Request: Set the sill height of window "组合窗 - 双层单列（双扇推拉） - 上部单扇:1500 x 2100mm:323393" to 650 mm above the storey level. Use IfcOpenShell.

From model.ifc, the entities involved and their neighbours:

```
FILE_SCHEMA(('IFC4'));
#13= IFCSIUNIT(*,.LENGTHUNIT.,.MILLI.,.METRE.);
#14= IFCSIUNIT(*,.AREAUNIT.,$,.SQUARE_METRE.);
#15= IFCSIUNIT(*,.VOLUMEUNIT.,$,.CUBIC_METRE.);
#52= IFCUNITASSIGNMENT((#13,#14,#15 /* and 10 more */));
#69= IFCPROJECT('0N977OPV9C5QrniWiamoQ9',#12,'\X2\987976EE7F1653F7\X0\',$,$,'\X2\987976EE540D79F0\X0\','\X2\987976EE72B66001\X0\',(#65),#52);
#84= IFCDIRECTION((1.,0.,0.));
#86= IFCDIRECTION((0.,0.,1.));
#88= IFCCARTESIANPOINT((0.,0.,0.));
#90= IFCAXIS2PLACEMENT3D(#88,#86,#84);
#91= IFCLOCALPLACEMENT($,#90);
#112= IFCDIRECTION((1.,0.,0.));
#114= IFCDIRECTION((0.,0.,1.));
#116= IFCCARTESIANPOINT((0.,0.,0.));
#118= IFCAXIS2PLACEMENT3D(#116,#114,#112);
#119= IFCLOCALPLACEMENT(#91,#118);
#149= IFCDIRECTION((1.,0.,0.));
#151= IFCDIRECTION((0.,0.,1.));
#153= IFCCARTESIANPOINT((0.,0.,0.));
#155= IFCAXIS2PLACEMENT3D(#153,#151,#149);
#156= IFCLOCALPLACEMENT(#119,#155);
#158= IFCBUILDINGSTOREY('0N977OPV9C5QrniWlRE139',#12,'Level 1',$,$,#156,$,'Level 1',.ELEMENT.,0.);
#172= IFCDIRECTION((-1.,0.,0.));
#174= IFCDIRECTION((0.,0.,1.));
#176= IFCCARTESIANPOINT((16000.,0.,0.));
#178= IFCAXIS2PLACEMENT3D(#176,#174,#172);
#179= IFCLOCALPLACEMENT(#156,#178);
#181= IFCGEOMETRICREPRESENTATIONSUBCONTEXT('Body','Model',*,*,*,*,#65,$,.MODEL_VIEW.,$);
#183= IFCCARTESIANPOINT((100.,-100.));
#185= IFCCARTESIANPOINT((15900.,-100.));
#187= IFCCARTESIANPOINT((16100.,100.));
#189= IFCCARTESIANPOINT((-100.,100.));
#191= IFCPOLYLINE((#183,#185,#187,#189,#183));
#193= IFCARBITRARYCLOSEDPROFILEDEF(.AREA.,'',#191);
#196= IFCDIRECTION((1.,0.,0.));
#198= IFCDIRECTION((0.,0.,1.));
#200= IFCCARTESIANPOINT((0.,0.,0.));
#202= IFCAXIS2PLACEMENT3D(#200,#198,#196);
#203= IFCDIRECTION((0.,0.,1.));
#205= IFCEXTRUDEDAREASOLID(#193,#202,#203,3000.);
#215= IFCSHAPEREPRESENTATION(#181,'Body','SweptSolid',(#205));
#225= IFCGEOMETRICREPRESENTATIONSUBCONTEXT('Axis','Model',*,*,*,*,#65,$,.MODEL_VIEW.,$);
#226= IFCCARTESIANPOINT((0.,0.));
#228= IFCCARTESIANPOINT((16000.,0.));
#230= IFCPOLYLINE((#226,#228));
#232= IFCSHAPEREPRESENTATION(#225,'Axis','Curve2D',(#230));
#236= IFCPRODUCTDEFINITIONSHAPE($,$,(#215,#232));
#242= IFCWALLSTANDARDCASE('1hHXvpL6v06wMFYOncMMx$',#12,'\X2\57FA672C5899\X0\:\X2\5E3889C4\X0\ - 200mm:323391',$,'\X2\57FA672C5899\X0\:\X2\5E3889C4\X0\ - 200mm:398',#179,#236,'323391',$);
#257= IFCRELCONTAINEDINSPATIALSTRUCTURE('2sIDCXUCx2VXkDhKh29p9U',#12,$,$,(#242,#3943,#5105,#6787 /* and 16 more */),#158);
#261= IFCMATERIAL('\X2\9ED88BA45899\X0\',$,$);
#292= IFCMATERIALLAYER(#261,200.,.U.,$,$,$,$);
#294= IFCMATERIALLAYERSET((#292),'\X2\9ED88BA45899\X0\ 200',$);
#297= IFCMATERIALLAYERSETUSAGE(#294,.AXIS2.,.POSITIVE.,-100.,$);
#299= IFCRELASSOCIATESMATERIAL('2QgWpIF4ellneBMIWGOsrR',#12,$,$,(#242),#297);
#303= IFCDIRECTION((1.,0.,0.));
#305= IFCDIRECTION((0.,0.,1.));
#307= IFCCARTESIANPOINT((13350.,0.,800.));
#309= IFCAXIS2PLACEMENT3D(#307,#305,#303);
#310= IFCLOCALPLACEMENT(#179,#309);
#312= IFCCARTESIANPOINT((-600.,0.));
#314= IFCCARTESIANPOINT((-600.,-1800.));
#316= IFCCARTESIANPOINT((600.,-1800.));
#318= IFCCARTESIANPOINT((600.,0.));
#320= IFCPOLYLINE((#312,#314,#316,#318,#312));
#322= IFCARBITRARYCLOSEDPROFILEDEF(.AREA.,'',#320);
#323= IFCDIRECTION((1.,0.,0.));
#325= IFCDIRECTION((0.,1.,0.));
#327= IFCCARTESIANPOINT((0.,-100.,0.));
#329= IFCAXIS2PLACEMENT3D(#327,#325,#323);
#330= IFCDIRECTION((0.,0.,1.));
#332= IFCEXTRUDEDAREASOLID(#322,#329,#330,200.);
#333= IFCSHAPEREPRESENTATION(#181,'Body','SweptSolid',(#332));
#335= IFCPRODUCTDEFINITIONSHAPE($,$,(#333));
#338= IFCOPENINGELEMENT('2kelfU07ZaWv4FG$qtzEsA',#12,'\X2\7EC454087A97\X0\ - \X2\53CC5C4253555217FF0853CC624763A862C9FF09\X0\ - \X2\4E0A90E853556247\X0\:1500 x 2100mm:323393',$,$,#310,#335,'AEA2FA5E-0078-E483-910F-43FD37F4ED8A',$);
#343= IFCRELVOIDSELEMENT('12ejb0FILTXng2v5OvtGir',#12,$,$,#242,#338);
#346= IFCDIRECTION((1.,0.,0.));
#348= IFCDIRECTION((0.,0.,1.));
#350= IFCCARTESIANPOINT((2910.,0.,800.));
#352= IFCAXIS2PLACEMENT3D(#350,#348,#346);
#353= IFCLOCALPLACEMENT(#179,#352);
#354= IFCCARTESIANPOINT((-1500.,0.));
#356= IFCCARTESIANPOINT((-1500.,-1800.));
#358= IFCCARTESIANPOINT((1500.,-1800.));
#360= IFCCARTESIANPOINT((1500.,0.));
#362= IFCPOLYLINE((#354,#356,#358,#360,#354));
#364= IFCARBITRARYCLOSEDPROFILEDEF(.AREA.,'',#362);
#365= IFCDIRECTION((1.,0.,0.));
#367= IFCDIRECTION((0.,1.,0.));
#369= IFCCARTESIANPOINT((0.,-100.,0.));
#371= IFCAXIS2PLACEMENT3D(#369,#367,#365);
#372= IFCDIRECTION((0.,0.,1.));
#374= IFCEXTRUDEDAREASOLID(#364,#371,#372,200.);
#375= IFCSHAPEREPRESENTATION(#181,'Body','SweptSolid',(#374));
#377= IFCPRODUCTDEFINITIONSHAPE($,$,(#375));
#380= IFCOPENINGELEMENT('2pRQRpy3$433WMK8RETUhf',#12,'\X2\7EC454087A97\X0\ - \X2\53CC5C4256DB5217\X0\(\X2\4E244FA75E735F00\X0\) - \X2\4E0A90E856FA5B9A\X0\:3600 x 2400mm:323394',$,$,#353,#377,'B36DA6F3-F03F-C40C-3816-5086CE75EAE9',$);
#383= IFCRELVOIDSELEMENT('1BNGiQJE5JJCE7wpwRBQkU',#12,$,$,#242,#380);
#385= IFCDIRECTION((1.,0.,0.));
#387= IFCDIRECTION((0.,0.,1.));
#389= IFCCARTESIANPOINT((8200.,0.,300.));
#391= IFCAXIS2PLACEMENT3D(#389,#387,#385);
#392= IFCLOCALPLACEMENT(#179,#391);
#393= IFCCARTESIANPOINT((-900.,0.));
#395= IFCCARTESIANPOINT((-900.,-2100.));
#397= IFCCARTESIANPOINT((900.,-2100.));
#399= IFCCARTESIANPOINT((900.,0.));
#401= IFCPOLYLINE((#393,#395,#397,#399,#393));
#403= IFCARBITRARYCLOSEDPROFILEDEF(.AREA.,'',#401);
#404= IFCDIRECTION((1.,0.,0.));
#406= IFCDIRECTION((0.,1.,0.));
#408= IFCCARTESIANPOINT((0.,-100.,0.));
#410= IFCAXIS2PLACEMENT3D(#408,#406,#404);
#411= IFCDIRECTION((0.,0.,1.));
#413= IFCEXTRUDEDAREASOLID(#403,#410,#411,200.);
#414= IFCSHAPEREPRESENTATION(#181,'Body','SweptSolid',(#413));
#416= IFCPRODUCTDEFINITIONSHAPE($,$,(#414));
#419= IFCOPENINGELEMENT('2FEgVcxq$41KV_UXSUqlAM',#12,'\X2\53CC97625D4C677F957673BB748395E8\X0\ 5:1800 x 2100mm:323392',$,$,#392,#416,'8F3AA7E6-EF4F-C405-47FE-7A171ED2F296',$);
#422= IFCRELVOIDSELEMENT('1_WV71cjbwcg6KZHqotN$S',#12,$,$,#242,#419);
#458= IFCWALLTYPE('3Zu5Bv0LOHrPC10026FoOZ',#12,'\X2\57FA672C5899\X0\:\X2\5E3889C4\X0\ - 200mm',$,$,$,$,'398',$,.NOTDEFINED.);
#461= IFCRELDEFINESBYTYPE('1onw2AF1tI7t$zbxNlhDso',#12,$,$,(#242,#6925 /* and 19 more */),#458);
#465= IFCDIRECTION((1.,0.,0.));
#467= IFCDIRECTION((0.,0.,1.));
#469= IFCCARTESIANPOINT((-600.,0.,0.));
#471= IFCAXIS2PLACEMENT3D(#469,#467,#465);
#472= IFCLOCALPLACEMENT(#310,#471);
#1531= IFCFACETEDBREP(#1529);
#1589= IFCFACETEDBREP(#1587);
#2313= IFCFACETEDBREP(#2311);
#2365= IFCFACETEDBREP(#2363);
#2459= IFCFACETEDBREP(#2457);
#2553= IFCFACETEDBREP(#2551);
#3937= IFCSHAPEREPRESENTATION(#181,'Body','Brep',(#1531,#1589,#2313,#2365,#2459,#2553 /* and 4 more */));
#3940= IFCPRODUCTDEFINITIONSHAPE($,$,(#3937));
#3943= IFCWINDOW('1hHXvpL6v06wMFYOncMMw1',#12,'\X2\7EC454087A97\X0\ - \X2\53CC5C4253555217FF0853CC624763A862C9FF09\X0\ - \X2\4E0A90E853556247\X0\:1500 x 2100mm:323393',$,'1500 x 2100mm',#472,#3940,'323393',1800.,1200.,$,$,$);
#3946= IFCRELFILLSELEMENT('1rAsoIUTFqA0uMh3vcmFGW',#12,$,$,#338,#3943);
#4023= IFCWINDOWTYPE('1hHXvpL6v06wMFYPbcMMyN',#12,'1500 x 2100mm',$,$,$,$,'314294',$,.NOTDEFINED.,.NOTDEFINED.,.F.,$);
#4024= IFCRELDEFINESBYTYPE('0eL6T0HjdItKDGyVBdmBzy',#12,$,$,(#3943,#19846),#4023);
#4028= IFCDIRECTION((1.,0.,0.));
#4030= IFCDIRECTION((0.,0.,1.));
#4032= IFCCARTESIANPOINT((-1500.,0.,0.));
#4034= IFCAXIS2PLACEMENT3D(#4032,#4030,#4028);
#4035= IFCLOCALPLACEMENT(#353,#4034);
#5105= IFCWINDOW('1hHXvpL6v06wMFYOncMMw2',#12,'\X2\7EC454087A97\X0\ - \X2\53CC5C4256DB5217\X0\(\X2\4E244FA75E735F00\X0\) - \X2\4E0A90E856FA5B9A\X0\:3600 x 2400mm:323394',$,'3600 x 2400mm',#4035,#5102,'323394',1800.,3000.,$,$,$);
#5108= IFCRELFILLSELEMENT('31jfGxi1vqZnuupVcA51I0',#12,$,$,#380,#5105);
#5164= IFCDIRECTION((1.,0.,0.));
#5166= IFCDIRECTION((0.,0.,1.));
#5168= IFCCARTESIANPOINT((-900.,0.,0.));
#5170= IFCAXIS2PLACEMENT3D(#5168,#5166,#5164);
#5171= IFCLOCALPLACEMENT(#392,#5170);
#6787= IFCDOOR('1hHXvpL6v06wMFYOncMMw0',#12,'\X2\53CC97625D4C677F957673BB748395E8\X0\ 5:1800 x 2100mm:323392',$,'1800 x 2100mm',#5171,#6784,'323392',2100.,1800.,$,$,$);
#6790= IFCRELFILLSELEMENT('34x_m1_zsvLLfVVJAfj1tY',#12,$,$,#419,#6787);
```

```python
import numpy as np
import ifcopenshell
import ifcopenshell.api.geometry
import ifcopenshell.geom
import ifcopenshell.util.element
import ifcopenshell.util.placement
import ifcopenshell.util.shape
import ifcopenshell.util.unit

model = ifcopenshell.open("model.ifc")
unit_scale = ifcopenshell.util.unit.calculate_unit_scale(model)

window = model.by_guid("1hHXvpL6v06wMFYOncMMw1")
opening = window.FillsVoids[0].RelatingOpeningElement
storey = ifcopenshell.util.element.get_container(window, ifc_class="IfcBuildingStorey")
level = ifcopenshell.util.placement.get_local_placement(storey.ObjectPlacement)[2, 3]

# The opening's origin need not be at the sill, so measure its lowest point.
shape = ifcopenshell.geom.create_shape(ifcopenshell.geom.settings(), opening)
bottom = ifcopenshell.util.shape.get_shape_bottom_elevation(shape, shape.geometry) / unit_scale
dz = level + 0.65 / unit_scale - bottom

shift = np.array([0.0, 0.0, dz])
# The window is placed relative to its opening, so it follows when the opening moves.
matrix = ifcopenshell.util.placement.get_local_placement(opening.ObjectPlacement)
matrix[:3, 3] += shift
ifcopenshell.api.geometry.edit_object_placement(
    model, product=opening, matrix=matrix, is_si=False, should_transform_children=True
)

print(f"moved by {dz * unit_scale:+.3f} m")

model.write("model_updated.ifc")
```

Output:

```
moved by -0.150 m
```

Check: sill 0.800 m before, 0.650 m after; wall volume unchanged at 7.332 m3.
